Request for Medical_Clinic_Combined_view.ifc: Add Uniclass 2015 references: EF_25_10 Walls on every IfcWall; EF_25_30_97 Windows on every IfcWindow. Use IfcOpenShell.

First a look at what the model holds.

```python
import ifcopenshell

model = ifcopenshell.open("Medical_Clinic_Combined_view.ifc")
print(model.schema)
print("classifications:", [c.Name for c in model.by_type("IfcClassification")])
for ifc_class in ("IfcDoor", "IfcRoof", "IfcStair", "IfcWall", "IfcWindow"):
    print(ifc_class, len(model.by_type(ifc_class)))
```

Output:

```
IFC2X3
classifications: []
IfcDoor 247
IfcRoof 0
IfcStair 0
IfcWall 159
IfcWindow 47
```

```python
import ifcopenshell
import ifcopenshell.api.classification

model = ifcopenshell.open("Medical_Clinic_Combined_view.ifc")

# IFC2X3 requires Source and Edition and has no link from the project to the system.
system = model.create_entity("IfcClassification", Source="NBS", Edition="2015", Name="Uniclass 2015")

codes = {
    "IfcWall": ("EF_25_10", "Walls"),
    "IfcWindow": ("EF_25_30_97", "Windows"),
}
for ifc_class, (code, name) in codes.items():
    products = model.by_type(ifc_class)
    ifcopenshell.api.classification.add_reference(
        model, products=products, classification=system, identification=code, name=name
    )
    print(code, len(products))

model.write("Medical_Clinic_Combined_view-out.ifc")
```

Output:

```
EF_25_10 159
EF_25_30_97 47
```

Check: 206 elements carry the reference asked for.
